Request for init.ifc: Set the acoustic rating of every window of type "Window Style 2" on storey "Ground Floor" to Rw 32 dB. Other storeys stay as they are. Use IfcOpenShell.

First a look at what the model holds.

```python
import ifcopenshell
import ifcopenshell.util.element

model = ifcopenshell.open("init.ifc")
print(model.schema)
storey = next(s for s in model.by_type("IfcBuildingStorey") if s.Name == "Ground Floor")
windows = [e for e in ifcopenshell.util.element.get_decomposition(storey) if e.is_a("IfcWindow")]
seen = {}
for e in windows:
    element_type = ifcopenshell.util.element.get_type(e)
    key = (element_type.Name if element_type != e and element_type else None, ifcopenshell.util.element.get_pset(e, "Pset_WindowCommon", "AcousticRating"))
    seen[key] = seen.get(key, 0) + 1
for (name, value), count in sorted(seen.items(), key=str):
    print(count, "x", name, "|", value)
```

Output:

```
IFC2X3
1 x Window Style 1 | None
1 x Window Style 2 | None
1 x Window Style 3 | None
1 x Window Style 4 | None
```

```python
import ifcopenshell
import ifcopenshell.api.pset
import ifcopenshell.util.element

model = ifcopenshell.open("init.ifc")

storey = next(s for s in model.by_type("IfcBuildingStorey") if s.Name == "Ground Floor")
windows = [e for e in ifcopenshell.util.element.get_decomposition(storey) if e.is_a("IfcWindow")]

count = 0
for e in windows:
    element_type = ifcopenshell.util.element.get_type(e)
    if element_type in (None, e) or element_type.Name != "Window Style 2":
        continue
    # add_pset returns the element's existing set when there is one.
    pset = ifcopenshell.api.pset.add_pset(model, product=e, name="Pset_WindowCommon")
    ifcopenshell.api.pset.edit_pset(model, pset=pset, properties={"AcousticRating": "Rw 32 dB"})
    count += 1

print(count, "windows updated")

model.write("init_updated.ifc")
```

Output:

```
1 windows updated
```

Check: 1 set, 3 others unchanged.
